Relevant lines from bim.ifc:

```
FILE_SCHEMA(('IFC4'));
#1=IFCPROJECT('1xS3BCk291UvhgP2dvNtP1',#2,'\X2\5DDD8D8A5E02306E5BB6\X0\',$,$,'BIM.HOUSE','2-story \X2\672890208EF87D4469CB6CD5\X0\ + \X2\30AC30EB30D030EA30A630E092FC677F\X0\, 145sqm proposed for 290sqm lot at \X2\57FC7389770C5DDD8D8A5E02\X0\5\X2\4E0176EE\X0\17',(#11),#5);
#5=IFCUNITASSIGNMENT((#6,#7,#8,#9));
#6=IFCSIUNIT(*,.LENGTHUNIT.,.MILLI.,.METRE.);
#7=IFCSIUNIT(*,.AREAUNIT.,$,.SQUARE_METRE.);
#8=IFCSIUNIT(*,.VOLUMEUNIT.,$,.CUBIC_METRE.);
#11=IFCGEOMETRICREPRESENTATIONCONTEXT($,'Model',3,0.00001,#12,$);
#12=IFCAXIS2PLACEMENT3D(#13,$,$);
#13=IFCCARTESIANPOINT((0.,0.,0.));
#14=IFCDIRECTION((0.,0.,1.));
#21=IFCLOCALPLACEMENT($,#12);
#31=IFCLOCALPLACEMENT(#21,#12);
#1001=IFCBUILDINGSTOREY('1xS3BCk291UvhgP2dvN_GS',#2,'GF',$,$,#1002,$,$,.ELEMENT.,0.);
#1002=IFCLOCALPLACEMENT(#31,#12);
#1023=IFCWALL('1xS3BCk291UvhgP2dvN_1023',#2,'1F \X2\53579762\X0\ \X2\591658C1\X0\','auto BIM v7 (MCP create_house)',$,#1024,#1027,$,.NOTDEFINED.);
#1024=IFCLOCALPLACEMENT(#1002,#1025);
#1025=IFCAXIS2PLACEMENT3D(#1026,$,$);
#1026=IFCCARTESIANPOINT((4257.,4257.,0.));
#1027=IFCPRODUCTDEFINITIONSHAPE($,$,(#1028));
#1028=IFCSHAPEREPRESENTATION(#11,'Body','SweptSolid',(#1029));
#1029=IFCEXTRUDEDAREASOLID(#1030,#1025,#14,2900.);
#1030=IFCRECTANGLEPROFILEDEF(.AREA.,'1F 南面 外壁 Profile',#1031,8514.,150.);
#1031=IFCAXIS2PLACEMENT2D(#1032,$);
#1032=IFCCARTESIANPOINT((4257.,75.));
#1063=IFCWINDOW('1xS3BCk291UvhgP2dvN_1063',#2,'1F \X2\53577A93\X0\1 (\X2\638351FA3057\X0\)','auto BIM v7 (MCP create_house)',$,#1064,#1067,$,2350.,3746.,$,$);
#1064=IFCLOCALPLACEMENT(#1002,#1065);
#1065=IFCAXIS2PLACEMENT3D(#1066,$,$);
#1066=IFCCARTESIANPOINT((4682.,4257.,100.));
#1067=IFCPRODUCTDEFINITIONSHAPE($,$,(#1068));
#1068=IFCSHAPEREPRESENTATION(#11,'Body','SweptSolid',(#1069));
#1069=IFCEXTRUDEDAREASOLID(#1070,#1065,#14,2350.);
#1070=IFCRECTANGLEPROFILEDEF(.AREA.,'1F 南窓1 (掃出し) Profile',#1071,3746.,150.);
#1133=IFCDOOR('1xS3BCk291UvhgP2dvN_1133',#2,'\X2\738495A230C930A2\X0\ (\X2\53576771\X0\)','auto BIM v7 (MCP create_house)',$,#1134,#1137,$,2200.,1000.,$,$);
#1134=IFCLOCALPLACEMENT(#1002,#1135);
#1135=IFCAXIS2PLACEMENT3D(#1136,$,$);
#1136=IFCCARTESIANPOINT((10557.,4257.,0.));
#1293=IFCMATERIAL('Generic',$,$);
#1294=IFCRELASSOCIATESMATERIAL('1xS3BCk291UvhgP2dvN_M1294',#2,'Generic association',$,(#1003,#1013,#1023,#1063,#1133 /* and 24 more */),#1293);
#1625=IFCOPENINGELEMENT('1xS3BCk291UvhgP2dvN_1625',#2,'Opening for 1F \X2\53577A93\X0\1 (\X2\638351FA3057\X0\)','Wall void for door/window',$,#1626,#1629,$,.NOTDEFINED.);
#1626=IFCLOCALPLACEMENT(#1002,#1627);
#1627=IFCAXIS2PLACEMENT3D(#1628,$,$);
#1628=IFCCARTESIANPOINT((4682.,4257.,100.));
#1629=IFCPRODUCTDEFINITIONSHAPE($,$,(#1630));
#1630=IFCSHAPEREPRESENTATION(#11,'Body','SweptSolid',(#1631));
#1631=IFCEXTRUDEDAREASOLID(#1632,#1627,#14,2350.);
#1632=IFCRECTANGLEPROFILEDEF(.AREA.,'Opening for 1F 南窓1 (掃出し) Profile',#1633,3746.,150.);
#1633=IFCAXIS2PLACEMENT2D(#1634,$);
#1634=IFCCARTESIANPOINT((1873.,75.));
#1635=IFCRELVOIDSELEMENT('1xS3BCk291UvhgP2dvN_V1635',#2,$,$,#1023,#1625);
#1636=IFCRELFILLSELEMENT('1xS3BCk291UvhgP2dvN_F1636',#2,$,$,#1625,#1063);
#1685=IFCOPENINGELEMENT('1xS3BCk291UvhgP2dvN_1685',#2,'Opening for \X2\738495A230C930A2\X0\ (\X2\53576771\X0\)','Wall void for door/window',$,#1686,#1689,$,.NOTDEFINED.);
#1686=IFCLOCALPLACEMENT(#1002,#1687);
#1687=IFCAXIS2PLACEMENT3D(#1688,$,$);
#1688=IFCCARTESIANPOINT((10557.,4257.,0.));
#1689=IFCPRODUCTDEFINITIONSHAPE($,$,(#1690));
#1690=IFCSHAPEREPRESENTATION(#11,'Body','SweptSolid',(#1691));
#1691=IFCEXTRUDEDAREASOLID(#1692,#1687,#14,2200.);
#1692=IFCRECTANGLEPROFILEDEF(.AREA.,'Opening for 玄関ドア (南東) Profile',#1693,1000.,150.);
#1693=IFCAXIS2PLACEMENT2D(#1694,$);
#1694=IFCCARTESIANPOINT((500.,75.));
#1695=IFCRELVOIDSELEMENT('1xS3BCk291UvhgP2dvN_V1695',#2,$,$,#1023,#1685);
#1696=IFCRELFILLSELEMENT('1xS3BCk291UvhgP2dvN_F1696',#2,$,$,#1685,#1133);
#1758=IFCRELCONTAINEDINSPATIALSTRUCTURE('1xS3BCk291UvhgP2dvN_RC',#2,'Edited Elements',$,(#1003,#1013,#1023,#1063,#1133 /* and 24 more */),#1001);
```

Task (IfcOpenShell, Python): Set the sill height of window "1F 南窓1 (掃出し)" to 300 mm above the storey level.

```python
import numpy as np
import ifcopenshell
import ifcopenshell.api.geometry
import ifcopenshell.geom
import ifcopenshell.util.element
import ifcopenshell.util.placement
import ifcopenshell.util.shape
import ifcopenshell.util.unit

model = ifcopenshell.open("bim.ifc")
unit_scale = ifcopenshell.util.unit.calculate_unit_scale(model)

window = model.by_guid("1xS3BCk291UvhgP2dvN_1063")
opening = window.FillsVoids[0].RelatingOpeningElement
storey = ifcopenshell.util.element.get_container(window, ifc_class="IfcBuildingStorey")
level = ifcopenshell.util.placement.get_local_placement(storey.ObjectPlacement)[2, 3]

# The opening's origin need not be at the sill, so measure its lowest point.
shape = ifcopenshell.geom.create_shape(ifcopenshell.geom.settings(), opening)
bottom = ifcopenshell.util.shape.get_shape_bottom_elevation(shape, shape.geometry) / unit_scale
dz = level + 0.3 / unit_scale - bottom

shift = np.array([0.0, 0.0, dz])
# The window is not placed relative to its opening, so move both.
for product in (opening, window):
    matrix = ifcopenshell.util.placement.get_local_placement(product.ObjectPlacement)
    matrix[:3, 3] += shift
    ifcopenshell.api.geometry.edit_object_placement(model, product=product, matrix=matrix, is_si=False)

print(f"moved by {dz * unit_scale:+.3f} m")

model.write("bim_updated.ifc")
```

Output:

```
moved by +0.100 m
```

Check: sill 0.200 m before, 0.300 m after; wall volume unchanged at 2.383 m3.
